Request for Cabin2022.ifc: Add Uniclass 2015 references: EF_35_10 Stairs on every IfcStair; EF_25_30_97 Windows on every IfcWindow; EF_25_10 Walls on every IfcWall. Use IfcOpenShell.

First a look at what the model holds.

```python
import ifcopenshell

model = ifcopenshell.open("Cabin2022.ifc")
print(model.schema)
print("classifications:", [c.Name for c in model.by_type("IfcClassification")])
for ifc_class in ("IfcDoor", "IfcRoof", "IfcStair", "IfcWall", "IfcWindow"):
    print(ifc_class, len(model.by_type(ifc_class)))
```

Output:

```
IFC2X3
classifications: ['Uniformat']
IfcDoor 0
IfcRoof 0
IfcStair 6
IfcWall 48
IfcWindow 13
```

```python
import ifcopenshell
import ifcopenshell.api.classification

model = ifcopenshell.open("Cabin2022.ifc")

# IFC2X3 requires Source and Edition and has no link from the project to the system.
system = model.create_entity("IfcClassification", Source="NBS", Edition="2015", Name="Uniclass 2015")

codes = {
    "IfcStair": ("EF_35_10", "Stairs"),
    "IfcWindow": ("EF_25_30_97", "Windows"),
    "IfcWall": ("EF_25_10", "Walls"),
}
for ifc_class, (code, name) in codes.items():
    products = model.by_type(ifc_class)
    ifcopenshell.api.classification.add_reference(
        model, products=products, classification=system, identification=code, name=name
    )
    print(code, len(products))

model.write("Cabin2022_edited.ifc")
```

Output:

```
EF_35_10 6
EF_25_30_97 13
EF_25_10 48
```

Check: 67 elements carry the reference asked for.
